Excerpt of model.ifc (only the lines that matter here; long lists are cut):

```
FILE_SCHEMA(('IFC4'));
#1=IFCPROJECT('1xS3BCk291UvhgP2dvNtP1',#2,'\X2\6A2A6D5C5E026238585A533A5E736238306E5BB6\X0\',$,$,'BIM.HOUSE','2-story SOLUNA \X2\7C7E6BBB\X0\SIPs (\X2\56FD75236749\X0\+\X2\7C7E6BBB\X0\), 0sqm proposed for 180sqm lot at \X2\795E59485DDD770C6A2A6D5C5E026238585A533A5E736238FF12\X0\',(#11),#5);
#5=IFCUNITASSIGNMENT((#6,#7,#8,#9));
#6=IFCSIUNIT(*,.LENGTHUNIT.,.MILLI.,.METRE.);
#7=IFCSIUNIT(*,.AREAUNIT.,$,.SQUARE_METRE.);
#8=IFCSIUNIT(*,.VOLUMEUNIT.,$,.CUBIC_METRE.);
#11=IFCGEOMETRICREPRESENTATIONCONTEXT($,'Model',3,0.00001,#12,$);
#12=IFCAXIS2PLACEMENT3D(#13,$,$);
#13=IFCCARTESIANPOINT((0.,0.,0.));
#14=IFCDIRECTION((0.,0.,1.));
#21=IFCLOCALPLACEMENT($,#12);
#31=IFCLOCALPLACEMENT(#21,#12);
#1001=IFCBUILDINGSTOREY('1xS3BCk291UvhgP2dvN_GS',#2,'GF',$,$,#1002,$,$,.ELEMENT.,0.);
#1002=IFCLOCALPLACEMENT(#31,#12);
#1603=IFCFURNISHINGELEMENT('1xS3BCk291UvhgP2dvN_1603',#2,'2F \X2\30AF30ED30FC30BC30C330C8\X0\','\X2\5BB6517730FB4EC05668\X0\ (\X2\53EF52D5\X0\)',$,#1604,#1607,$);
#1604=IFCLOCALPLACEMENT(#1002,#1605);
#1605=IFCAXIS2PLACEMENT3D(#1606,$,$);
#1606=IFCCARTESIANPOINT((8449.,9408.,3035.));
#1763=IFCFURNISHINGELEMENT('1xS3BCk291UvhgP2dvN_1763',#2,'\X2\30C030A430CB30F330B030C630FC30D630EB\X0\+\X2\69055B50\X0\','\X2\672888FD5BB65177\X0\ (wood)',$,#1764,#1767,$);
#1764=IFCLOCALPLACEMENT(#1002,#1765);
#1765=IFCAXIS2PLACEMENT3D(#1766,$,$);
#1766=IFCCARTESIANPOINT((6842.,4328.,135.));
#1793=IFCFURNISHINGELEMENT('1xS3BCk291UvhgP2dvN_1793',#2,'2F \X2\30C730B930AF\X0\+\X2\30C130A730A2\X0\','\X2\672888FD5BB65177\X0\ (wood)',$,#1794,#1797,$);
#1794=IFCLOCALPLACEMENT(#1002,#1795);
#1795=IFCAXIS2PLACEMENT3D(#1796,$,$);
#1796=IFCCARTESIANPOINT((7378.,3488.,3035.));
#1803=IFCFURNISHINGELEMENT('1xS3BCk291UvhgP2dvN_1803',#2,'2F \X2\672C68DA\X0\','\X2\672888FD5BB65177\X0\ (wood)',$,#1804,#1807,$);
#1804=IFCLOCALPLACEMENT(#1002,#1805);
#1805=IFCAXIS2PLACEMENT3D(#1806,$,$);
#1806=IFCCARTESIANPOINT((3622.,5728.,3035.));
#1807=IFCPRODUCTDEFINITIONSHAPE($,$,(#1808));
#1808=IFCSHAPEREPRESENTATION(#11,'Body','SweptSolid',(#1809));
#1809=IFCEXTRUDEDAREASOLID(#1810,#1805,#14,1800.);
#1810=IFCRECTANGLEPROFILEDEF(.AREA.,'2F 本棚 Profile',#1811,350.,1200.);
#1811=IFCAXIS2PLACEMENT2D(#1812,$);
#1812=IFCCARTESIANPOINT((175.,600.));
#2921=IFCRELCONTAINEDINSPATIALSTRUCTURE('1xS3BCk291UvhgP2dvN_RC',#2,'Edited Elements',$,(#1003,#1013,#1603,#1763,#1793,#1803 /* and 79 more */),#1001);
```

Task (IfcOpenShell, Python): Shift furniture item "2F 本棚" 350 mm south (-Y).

```python
import ifcopenshell
import ifcopenshell.api.geometry
import ifcopenshell.util.placement
import ifcopenshell.util.unit

model = ifcopenshell.open("model.ifc")
unit_scale = ifcopenshell.util.unit.calculate_unit_scale(model)

item = model.by_guid("1xS3BCk291UvhgP2dvN_1803")
matrix = ifcopenshell.util.placement.get_local_placement(item.ObjectPlacement)
matrix[1, 3] -= 0.35 / unit_scale
ifcopenshell.api.geometry.edit_object_placement(model, product=item, matrix=matrix, is_si=False)

print(ifcopenshell.util.placement.get_local_placement(item.ObjectPlacement).round(3) + 0.0)

model.write("model_updated.ifc")
```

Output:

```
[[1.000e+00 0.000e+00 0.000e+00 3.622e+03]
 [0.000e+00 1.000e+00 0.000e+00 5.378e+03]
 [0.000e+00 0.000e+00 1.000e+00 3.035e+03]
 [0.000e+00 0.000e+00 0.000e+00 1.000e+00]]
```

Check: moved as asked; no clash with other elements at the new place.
